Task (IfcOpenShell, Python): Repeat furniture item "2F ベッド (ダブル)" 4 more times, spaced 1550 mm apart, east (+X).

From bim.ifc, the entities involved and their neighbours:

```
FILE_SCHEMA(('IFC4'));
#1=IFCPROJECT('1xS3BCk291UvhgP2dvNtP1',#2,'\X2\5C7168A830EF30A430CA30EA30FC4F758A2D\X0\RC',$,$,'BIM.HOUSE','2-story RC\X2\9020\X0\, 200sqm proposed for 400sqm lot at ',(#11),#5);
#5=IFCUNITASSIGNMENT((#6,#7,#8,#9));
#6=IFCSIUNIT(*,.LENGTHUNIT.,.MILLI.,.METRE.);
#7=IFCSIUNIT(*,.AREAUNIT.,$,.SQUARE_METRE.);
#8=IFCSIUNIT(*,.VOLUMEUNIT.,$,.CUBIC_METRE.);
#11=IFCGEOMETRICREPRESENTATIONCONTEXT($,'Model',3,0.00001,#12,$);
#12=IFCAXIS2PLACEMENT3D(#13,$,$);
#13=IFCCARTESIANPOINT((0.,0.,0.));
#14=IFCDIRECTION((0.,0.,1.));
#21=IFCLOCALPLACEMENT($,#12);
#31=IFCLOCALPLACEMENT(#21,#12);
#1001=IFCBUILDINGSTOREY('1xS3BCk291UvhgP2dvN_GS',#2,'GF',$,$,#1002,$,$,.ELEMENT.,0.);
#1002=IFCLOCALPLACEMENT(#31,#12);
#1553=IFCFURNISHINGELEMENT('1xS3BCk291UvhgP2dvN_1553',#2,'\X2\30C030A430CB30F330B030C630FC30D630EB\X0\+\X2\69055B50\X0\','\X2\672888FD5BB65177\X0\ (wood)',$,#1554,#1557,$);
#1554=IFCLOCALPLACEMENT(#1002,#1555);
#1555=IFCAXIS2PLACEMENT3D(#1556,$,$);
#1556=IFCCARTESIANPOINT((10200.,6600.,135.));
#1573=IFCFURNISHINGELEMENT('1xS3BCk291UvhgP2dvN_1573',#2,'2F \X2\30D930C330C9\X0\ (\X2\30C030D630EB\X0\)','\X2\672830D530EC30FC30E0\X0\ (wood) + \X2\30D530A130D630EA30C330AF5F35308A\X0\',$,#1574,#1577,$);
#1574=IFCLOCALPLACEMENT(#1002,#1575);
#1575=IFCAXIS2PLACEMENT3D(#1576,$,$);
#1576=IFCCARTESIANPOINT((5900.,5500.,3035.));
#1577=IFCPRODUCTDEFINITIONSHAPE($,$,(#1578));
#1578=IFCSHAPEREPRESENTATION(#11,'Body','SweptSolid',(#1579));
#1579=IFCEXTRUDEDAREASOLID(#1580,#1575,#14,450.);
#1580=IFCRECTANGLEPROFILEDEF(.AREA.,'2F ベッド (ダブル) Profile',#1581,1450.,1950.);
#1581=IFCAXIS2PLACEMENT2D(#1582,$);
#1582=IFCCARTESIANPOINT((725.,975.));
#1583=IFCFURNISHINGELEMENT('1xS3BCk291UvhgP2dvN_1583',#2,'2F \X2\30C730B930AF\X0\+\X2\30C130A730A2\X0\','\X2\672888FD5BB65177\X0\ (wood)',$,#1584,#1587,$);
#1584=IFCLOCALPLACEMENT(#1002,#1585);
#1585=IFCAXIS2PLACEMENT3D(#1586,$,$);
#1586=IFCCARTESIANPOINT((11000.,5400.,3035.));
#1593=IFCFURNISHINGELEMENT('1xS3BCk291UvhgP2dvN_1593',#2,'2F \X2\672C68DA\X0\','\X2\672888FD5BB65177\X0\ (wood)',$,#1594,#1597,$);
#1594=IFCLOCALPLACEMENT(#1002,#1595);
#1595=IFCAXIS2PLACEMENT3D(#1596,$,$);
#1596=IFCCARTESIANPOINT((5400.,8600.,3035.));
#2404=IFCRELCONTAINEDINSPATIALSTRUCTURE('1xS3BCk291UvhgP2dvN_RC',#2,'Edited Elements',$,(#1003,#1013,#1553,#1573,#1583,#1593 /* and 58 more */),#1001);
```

```python
import numpy as np
import ifcopenshell
import ifcopenshell.api.geometry
import ifcopenshell.api.root
import ifcopenshell.util.element
import ifcopenshell.util.placement

model = ifcopenshell.open("bim.ifc")


def reuse_history(source, copy):
    """copy_class also copies each property set's owner history, people and application; keep the originals."""
    for rel in copy.IsDefinedBy:
        if rel.is_a("IfcRelDefinesByProperties") and (history := rel.RelatingPropertyDefinition.OwnerHistory):
            rel.RelatingPropertyDefinition.OwnerHistory = source.OwnerHistory
            ifcopenshell.util.element.remove_deep2(model, history)


source = model.by_guid("1xS3BCk291UvhgP2dvN_1573")
base = ifcopenshell.util.placement.get_local_placement(source.ObjectPlacement)
step = np.array([1.0, 0.0, 0.0]) * 1550.0

for i in range(1, 5):
    copy = ifcopenshell.api.root.copy_class(model, product=source)
    copy.Representation = ifcopenshell.util.element.copy_deep(
        model, source.Representation, exclude=["IfcGeometricRepresentationContext", "IfcRepresentationMap"]
    )
    reuse_history(source, copy)
    matrix = base.copy()
    matrix[:3, 3] += i * step
    print("added at", matrix[:3, 3].round(3) + 0.0)
    ifcopenshell.api.geometry.edit_object_placement(model, product=copy, matrix=matrix, is_si=False)

model.write("bim-out.ifc")
```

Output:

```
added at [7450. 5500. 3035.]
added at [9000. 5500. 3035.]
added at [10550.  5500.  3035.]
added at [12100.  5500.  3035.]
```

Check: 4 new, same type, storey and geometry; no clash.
